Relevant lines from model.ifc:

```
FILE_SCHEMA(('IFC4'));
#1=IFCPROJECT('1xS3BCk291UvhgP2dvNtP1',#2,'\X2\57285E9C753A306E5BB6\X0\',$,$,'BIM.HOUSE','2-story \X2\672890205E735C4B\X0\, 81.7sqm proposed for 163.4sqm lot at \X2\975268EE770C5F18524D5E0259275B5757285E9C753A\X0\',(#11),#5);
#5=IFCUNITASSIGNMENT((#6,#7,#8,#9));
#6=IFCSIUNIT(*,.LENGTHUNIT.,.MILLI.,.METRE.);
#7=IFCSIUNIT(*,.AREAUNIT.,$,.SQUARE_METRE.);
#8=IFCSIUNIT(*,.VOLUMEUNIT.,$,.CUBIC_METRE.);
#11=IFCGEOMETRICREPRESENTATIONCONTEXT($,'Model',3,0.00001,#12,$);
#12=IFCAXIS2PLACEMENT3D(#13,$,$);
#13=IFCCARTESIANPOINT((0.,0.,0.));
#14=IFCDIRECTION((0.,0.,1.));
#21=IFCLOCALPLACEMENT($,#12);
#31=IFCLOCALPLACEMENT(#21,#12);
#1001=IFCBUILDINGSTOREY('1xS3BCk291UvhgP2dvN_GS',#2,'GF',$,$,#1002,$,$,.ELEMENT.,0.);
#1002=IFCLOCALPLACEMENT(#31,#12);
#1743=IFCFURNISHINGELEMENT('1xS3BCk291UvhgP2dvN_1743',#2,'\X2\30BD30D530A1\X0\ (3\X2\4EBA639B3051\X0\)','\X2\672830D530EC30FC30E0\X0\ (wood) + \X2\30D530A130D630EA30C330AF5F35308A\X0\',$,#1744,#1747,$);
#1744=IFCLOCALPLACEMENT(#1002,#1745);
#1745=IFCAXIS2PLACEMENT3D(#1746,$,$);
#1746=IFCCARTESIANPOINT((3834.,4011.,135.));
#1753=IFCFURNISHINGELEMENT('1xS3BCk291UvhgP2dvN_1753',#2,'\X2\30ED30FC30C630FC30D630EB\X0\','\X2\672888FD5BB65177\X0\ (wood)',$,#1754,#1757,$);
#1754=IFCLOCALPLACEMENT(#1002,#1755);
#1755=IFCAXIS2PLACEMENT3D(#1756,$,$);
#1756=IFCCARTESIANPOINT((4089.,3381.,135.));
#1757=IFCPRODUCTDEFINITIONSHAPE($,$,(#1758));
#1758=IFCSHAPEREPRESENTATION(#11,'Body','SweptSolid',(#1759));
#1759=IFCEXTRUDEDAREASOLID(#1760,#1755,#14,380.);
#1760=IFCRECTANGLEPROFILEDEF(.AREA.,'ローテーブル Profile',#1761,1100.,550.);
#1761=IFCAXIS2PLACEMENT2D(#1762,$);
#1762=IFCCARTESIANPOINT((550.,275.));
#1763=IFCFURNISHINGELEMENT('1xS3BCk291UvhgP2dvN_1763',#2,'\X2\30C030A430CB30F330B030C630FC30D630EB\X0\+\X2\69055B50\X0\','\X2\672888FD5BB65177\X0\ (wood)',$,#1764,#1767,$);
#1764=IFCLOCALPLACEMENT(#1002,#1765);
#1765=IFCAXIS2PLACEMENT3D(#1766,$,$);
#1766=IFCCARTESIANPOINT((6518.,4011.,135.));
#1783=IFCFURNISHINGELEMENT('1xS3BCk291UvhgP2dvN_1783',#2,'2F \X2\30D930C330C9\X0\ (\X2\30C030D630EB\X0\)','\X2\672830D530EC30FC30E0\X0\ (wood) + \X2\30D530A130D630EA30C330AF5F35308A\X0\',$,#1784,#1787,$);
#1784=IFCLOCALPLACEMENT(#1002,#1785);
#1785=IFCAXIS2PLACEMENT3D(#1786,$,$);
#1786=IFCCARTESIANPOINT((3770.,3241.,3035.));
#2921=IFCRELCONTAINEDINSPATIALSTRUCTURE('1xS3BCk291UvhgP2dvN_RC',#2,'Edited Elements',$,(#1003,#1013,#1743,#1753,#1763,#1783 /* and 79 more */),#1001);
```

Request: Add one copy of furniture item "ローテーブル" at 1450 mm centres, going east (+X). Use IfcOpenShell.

```python
import numpy as np
import ifcopenshell
import ifcopenshell.api.geometry
import ifcopenshell.api.root
import ifcopenshell.util.element
import ifcopenshell.util.placement
import ifcopenshell.util.unit

model = ifcopenshell.open("model.ifc")
unit_scale = ifcopenshell.util.unit.calculate_unit_scale(model)


def reuse_history(source, copy):
    """copy_class also copies each property set's owner history, people and application; keep the originals."""
    for rel in copy.IsDefinedBy:
        if rel.is_a("IfcRelDefinesByProperties") and (history := rel.RelatingPropertyDefinition.OwnerHistory):
            rel.RelatingPropertyDefinition.OwnerHistory = source.OwnerHistory
            ifcopenshell.util.element.remove_deep2(model, history)


source = model.by_guid("1xS3BCk291UvhgP2dvN_1753")
base = ifcopenshell.util.placement.get_local_placement(source.ObjectPlacement)
step = np.array([1.0, 0.0, 0.0]) * 1.45 / unit_scale

for i in range(1, 2):
    copy = ifcopenshell.api.root.copy_class(model, product=source)
    copy.Representation = ifcopenshell.util.element.copy_deep(
        model, source.Representation, exclude=["IfcGeometricRepresentationContext", "IfcRepresentationMap"]
    )
    reuse_history(source, copy)
    matrix = base.copy()
    matrix[:3, 3] += i * step
    print("added at", matrix[:3, 3].round(3) + 0.0)
    ifcopenshell.api.geometry.edit_object_placement(model, product=copy, matrix=matrix, is_si=False)

model.write("model_edited.ifc")
```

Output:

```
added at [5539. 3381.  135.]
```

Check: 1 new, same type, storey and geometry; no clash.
